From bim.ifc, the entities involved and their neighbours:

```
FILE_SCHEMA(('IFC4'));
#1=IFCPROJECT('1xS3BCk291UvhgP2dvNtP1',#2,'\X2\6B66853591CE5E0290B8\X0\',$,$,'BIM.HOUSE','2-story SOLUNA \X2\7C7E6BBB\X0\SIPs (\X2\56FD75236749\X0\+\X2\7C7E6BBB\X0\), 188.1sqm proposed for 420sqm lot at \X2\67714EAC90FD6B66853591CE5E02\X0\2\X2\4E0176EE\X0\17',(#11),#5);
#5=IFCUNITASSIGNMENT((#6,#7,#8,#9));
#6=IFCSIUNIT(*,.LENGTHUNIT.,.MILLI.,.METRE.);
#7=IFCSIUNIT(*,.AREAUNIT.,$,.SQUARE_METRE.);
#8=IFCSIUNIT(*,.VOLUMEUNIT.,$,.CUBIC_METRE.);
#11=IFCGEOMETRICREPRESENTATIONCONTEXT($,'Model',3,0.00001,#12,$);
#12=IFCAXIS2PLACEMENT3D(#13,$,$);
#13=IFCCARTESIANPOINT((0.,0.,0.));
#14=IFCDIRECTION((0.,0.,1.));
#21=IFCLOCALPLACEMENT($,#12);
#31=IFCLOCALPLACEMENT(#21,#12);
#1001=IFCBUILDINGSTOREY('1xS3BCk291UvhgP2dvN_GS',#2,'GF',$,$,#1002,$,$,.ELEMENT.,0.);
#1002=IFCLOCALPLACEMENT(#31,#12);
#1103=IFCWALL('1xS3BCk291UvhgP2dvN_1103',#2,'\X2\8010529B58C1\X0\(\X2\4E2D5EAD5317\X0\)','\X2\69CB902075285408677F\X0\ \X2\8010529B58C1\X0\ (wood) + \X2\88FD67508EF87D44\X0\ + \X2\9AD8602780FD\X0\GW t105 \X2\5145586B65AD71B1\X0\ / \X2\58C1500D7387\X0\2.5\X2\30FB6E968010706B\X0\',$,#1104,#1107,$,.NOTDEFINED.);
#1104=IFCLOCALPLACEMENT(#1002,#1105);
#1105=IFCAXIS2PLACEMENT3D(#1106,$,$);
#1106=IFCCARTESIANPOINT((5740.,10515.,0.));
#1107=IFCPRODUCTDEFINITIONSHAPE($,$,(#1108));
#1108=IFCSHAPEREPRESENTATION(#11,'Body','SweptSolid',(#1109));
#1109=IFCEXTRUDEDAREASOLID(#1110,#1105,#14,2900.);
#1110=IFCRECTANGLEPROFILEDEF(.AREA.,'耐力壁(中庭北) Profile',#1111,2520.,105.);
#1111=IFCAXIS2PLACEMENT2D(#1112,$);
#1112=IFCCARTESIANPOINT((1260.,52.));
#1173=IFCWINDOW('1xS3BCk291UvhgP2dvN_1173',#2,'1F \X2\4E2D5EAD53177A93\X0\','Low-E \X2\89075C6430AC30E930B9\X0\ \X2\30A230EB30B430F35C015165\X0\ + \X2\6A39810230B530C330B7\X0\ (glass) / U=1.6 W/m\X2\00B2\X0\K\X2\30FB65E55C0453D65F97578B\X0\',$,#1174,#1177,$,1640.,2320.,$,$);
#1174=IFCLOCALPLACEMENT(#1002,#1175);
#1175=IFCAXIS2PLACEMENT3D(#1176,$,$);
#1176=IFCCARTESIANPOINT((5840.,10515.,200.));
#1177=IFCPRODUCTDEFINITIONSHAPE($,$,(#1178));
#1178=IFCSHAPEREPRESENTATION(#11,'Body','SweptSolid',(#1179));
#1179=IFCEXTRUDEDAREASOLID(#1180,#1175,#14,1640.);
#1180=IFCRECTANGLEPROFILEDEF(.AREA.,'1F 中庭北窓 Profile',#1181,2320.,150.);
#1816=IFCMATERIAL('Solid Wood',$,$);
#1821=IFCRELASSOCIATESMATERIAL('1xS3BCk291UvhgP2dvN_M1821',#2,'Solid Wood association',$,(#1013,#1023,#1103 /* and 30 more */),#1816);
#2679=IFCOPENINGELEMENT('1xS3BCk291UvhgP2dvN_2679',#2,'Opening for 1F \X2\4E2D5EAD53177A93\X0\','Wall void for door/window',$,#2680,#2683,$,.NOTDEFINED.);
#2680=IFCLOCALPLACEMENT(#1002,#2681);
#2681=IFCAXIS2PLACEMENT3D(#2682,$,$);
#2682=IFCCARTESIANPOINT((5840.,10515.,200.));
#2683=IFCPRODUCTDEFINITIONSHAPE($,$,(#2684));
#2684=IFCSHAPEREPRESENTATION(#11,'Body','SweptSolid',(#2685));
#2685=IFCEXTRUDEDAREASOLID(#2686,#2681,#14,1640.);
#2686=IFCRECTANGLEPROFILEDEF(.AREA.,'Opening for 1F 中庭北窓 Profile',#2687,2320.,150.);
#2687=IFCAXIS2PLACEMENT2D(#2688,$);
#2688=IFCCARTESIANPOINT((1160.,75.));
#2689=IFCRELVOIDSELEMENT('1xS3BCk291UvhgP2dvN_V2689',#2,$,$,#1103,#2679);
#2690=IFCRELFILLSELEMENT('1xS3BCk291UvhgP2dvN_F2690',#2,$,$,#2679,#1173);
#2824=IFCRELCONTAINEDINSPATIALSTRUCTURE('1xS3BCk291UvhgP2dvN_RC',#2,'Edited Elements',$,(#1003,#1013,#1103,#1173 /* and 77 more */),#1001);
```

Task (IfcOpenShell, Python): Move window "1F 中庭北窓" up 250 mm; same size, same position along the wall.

```python
import numpy as np
import ifcopenshell
import ifcopenshell.api.geometry
import ifcopenshell.util.placement
import ifcopenshell.util.unit

model = ifcopenshell.open("bim.ifc")
unit_scale = ifcopenshell.util.unit.calculate_unit_scale(model)

window = model.by_id(1173)
opening = window.FillsVoids[0].RelatingOpeningElement
dz = 250.0

shift = np.array([0.0, 0.0, dz])
# The window is not placed relative to its opening, so move both.
for product in (opening, window):
    matrix = ifcopenshell.util.placement.get_local_placement(product.ObjectPlacement)
    matrix[:3, 3] += shift
    ifcopenshell.api.geometry.edit_object_placement(model, product=product, matrix=matrix, is_si=False)

print(f"moved by {dz * unit_scale:+.3f} m")

model.write("bim-out.ifc")
```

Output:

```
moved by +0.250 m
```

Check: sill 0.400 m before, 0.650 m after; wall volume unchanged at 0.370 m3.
